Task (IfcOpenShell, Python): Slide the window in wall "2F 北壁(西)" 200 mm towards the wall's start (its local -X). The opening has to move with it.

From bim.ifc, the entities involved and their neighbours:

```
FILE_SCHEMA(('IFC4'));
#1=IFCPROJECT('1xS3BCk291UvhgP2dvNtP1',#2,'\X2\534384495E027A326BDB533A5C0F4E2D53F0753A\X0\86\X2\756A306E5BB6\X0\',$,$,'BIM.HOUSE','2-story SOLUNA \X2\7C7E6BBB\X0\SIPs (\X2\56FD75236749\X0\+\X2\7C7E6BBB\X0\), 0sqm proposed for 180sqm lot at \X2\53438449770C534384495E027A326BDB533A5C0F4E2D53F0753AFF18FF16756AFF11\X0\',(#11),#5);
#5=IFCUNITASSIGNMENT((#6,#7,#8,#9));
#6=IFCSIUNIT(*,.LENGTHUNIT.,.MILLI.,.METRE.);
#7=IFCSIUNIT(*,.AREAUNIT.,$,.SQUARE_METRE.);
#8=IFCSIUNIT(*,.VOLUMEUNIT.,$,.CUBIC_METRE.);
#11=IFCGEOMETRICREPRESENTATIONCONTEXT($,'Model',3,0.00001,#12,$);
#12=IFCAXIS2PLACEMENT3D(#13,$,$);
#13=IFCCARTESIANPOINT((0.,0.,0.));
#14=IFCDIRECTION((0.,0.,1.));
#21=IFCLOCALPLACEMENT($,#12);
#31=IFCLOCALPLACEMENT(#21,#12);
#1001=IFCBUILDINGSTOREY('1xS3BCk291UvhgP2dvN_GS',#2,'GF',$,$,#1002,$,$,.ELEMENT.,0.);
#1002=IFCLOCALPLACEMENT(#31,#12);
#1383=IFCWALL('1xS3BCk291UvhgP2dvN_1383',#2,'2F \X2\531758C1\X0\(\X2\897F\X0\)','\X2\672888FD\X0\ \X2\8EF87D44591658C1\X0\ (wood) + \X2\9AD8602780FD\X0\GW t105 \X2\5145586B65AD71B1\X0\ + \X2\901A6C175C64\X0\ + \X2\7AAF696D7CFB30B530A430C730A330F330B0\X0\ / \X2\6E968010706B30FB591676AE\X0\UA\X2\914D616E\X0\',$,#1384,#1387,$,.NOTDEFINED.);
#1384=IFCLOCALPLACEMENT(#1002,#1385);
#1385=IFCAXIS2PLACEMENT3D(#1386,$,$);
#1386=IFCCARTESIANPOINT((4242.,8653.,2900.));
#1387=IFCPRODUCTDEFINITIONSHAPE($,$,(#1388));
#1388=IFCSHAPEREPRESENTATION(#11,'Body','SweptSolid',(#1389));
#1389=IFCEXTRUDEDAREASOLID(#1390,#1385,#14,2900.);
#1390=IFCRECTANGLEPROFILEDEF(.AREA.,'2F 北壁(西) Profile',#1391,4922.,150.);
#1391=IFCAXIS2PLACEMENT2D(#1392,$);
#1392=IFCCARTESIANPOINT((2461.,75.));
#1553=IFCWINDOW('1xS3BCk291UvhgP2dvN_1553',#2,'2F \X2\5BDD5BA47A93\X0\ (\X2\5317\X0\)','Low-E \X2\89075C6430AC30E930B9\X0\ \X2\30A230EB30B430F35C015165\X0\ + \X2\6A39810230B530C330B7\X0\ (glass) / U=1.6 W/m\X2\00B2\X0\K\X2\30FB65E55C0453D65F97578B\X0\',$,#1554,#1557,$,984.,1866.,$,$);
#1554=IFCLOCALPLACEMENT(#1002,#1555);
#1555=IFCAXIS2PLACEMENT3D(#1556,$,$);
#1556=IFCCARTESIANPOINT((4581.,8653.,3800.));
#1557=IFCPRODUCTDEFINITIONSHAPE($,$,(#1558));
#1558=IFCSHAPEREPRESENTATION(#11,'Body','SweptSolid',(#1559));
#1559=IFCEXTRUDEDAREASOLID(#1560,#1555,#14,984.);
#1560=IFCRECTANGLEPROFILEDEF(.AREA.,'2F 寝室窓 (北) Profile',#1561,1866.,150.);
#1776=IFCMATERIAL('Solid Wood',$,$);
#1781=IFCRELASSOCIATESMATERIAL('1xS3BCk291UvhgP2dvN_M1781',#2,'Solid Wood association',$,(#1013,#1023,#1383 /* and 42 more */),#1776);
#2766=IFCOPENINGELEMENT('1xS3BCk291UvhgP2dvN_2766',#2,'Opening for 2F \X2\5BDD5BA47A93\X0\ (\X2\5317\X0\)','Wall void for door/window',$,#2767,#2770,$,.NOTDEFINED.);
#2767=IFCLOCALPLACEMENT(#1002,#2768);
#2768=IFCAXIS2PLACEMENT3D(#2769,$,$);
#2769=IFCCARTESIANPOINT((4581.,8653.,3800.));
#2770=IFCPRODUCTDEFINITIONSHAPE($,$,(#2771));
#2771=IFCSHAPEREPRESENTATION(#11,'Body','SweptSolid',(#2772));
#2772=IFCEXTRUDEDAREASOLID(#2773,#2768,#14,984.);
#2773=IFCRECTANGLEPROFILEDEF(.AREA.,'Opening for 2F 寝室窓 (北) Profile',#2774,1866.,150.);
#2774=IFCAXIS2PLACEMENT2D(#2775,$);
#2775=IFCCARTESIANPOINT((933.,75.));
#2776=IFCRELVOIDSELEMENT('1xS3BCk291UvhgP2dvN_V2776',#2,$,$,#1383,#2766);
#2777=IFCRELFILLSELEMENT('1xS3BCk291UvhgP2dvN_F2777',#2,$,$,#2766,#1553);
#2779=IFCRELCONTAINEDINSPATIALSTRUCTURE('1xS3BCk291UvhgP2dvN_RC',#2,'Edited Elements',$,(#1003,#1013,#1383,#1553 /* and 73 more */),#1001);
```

```python
import ifcopenshell
import ifcopenshell.api.geometry
import ifcopenshell.util.placement
import ifcopenshell.util.unit

model = ifcopenshell.open("bim.ifc")
unit_scale = ifcopenshell.util.unit.calculate_unit_scale(model)

window = model.by_guid("1xS3BCk291UvhgP2dvN_1553")
opening = window.FillsVoids[0].RelatingOpeningElement
wall = opening.VoidsElements[0].RelatingBuildingElement

wall_matrix = ifcopenshell.util.placement.get_local_placement(wall.ObjectPlacement)
shift = wall_matrix[:3, 0] * -0.2 / unit_scale
before = ifcopenshell.util.placement.get_local_placement(window.ObjectPlacement)[:3, 3].copy()

# The window is not placed relative to its opening, so move both.
for product in (opening, window):
    matrix = ifcopenshell.util.placement.get_local_placement(product.ObjectPlacement)
    matrix[:3, 3] += shift
    ifcopenshell.api.geometry.edit_object_placement(model, product=product, matrix=matrix, is_si=False)

after = ifcopenshell.util.placement.get_local_placement(window.ObjectPlacement)[:3, 3]
print("window moved by", (after - before).round(3) + 0.0)

model.write("bim_rev.ifc")
```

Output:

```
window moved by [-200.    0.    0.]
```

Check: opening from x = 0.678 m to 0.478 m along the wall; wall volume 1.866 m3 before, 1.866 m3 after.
